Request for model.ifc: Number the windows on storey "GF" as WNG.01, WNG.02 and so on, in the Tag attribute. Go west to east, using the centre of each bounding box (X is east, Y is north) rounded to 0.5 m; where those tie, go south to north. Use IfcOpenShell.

First a look at what the model holds.

```python
import ifcopenshell
import ifcopenshell.util.element
import ifcopenshell.util.placement

model = ifcopenshell.open("model.ifc")
print(model.schema)
storey = next(s for s in model.by_type("IfcBuildingStorey") if s.Name == "GF")
windows = [e for e in ifcopenshell.util.element.get_decomposition(storey) if e.is_a("IfcWindow")]
for e in sorted(windows, key=lambda e: e.id()):
    origin = ifcopenshell.util.placement.get_local_placement(e.ObjectPlacement)[:3, 3]
    print(e.id(), e.Tag, e.Name, origin.round(2) + 0.0, sep=" | ")
```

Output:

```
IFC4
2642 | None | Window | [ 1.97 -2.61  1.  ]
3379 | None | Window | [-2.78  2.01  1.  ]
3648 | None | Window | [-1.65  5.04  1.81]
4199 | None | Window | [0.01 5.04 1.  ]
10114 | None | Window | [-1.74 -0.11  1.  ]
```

```python
import ifcopenshell
import ifcopenshell.geom
import ifcopenshell.util.element
import ifcopenshell.util.shape

model = ifcopenshell.open("model.ifc")
settings = ifcopenshell.geom.settings()
settings.set("use-world-coords", True)


def centre(element):
    shape = ifcopenshell.geom.create_shape(settings, element)
    return ifcopenshell.util.shape.get_bbox_centroid(shape.geometry)


storey = next(s for s in model.by_type("IfcBuildingStorey") if s.Name == "GF")
windows = [e for e in ifcopenshell.util.element.get_decomposition(storey) if e.is_a("IfcWindow")]

# Insertion points can sit at a corner or the storey origin, so sort by the geometry (in metres).
centres = {e: centre(e) for e in windows}
windows.sort(key=lambda e: (round(centres[e][0] / 0.5), centres[e][1]))

for i, e in enumerate(windows, start=1):
    number = f"WNG.{i:02d}"
    e.Tag = number
    print(e.id(), number)

model.write("model-out.ifc")
```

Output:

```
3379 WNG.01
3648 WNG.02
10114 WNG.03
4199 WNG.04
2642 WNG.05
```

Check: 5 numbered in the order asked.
